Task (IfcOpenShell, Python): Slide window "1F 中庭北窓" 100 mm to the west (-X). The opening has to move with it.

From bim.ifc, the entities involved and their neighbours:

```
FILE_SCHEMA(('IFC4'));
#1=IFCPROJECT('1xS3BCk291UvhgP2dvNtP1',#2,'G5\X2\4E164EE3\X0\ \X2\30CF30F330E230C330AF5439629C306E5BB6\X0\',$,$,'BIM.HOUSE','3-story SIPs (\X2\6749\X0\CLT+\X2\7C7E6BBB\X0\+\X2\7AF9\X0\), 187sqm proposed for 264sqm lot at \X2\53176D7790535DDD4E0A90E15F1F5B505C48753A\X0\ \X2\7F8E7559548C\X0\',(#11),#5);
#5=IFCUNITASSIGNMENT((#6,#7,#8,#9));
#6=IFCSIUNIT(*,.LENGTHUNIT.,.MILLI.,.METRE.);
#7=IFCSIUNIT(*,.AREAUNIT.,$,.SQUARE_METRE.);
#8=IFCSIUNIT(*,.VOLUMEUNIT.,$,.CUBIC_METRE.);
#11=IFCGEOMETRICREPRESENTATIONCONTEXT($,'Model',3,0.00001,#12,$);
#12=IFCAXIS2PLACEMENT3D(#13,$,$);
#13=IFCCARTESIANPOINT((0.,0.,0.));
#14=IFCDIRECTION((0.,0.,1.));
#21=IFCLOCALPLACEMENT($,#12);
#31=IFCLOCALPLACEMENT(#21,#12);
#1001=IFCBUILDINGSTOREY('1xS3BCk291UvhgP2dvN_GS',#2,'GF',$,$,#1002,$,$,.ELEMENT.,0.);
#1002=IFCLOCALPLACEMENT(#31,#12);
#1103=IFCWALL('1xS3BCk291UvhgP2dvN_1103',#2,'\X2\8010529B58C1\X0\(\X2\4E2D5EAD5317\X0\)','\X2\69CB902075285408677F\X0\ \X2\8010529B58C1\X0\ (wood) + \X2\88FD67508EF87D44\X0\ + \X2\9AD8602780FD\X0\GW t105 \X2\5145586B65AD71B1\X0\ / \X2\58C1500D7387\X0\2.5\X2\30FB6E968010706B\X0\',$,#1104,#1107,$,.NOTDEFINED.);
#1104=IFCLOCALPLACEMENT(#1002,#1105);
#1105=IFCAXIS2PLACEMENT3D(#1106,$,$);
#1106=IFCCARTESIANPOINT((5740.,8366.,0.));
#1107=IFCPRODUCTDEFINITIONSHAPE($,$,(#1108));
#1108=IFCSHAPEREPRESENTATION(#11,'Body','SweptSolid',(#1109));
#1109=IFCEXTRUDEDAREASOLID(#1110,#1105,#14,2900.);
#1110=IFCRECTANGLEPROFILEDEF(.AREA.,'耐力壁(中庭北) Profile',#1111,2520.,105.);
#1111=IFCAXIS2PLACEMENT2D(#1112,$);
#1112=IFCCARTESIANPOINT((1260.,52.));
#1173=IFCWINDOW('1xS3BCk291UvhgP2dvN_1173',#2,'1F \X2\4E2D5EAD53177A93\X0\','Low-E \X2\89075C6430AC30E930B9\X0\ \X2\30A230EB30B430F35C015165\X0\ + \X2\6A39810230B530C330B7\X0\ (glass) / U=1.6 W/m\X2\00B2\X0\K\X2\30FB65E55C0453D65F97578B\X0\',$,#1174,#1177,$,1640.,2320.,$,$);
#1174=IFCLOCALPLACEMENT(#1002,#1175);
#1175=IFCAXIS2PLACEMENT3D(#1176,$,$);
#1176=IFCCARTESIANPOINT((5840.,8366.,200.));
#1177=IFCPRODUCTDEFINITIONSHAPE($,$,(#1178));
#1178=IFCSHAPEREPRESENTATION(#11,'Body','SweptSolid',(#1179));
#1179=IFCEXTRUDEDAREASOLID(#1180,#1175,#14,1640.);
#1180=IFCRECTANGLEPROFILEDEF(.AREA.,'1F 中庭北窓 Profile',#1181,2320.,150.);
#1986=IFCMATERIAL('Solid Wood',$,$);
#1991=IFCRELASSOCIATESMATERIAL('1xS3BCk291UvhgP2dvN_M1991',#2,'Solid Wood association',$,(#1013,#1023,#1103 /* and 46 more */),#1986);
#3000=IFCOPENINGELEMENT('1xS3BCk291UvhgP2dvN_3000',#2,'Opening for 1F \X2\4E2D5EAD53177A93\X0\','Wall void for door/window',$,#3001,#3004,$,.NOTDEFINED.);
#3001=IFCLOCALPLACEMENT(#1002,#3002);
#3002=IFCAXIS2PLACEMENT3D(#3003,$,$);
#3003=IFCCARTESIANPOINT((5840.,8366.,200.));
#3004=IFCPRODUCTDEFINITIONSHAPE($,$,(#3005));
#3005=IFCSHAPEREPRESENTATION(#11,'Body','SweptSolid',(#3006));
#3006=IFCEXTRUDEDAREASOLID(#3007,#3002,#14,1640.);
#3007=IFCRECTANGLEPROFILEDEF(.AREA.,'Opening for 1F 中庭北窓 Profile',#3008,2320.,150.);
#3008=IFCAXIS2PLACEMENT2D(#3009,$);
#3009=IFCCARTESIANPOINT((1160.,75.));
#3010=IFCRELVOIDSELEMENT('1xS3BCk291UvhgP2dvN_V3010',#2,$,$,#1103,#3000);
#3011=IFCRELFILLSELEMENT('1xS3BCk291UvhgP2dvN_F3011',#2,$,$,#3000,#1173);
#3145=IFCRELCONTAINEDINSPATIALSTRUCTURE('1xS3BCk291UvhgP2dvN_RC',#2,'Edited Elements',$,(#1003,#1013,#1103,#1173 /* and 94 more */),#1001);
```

```python
import ifcopenshell
import ifcopenshell.api.geometry
import ifcopenshell.util.placement

model = ifcopenshell.open("bim.ifc")

window = model.by_guid("1xS3BCk291UvhgP2dvN_1173")
opening = window.FillsVoids[0].RelatingOpeningElement
wall = opening.VoidsElements[0].RelatingBuildingElement

wall_matrix = ifcopenshell.util.placement.get_local_placement(wall.ObjectPlacement)
shift = wall_matrix[:3, 0] * -100.0
before = ifcopenshell.util.placement.get_local_placement(window.ObjectPlacement)[:3, 3].copy()

# The window is not placed relative to its opening, so move both.
for product in (opening, window):
    matrix = ifcopenshell.util.placement.get_local_placement(product.ObjectPlacement)
    matrix[:3, 3] += shift
    ifcopenshell.api.geometry.edit_object_placement(model, product=product, matrix=matrix, is_si=False)

after = ifcopenshell.util.placement.get_local_placement(window.ObjectPlacement)[:3, 3]
print("window moved by", (after - before).round(3) + 0.0)

model.write("bim_rev.ifc")
```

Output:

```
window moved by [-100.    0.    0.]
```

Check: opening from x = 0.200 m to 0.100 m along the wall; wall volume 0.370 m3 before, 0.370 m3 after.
